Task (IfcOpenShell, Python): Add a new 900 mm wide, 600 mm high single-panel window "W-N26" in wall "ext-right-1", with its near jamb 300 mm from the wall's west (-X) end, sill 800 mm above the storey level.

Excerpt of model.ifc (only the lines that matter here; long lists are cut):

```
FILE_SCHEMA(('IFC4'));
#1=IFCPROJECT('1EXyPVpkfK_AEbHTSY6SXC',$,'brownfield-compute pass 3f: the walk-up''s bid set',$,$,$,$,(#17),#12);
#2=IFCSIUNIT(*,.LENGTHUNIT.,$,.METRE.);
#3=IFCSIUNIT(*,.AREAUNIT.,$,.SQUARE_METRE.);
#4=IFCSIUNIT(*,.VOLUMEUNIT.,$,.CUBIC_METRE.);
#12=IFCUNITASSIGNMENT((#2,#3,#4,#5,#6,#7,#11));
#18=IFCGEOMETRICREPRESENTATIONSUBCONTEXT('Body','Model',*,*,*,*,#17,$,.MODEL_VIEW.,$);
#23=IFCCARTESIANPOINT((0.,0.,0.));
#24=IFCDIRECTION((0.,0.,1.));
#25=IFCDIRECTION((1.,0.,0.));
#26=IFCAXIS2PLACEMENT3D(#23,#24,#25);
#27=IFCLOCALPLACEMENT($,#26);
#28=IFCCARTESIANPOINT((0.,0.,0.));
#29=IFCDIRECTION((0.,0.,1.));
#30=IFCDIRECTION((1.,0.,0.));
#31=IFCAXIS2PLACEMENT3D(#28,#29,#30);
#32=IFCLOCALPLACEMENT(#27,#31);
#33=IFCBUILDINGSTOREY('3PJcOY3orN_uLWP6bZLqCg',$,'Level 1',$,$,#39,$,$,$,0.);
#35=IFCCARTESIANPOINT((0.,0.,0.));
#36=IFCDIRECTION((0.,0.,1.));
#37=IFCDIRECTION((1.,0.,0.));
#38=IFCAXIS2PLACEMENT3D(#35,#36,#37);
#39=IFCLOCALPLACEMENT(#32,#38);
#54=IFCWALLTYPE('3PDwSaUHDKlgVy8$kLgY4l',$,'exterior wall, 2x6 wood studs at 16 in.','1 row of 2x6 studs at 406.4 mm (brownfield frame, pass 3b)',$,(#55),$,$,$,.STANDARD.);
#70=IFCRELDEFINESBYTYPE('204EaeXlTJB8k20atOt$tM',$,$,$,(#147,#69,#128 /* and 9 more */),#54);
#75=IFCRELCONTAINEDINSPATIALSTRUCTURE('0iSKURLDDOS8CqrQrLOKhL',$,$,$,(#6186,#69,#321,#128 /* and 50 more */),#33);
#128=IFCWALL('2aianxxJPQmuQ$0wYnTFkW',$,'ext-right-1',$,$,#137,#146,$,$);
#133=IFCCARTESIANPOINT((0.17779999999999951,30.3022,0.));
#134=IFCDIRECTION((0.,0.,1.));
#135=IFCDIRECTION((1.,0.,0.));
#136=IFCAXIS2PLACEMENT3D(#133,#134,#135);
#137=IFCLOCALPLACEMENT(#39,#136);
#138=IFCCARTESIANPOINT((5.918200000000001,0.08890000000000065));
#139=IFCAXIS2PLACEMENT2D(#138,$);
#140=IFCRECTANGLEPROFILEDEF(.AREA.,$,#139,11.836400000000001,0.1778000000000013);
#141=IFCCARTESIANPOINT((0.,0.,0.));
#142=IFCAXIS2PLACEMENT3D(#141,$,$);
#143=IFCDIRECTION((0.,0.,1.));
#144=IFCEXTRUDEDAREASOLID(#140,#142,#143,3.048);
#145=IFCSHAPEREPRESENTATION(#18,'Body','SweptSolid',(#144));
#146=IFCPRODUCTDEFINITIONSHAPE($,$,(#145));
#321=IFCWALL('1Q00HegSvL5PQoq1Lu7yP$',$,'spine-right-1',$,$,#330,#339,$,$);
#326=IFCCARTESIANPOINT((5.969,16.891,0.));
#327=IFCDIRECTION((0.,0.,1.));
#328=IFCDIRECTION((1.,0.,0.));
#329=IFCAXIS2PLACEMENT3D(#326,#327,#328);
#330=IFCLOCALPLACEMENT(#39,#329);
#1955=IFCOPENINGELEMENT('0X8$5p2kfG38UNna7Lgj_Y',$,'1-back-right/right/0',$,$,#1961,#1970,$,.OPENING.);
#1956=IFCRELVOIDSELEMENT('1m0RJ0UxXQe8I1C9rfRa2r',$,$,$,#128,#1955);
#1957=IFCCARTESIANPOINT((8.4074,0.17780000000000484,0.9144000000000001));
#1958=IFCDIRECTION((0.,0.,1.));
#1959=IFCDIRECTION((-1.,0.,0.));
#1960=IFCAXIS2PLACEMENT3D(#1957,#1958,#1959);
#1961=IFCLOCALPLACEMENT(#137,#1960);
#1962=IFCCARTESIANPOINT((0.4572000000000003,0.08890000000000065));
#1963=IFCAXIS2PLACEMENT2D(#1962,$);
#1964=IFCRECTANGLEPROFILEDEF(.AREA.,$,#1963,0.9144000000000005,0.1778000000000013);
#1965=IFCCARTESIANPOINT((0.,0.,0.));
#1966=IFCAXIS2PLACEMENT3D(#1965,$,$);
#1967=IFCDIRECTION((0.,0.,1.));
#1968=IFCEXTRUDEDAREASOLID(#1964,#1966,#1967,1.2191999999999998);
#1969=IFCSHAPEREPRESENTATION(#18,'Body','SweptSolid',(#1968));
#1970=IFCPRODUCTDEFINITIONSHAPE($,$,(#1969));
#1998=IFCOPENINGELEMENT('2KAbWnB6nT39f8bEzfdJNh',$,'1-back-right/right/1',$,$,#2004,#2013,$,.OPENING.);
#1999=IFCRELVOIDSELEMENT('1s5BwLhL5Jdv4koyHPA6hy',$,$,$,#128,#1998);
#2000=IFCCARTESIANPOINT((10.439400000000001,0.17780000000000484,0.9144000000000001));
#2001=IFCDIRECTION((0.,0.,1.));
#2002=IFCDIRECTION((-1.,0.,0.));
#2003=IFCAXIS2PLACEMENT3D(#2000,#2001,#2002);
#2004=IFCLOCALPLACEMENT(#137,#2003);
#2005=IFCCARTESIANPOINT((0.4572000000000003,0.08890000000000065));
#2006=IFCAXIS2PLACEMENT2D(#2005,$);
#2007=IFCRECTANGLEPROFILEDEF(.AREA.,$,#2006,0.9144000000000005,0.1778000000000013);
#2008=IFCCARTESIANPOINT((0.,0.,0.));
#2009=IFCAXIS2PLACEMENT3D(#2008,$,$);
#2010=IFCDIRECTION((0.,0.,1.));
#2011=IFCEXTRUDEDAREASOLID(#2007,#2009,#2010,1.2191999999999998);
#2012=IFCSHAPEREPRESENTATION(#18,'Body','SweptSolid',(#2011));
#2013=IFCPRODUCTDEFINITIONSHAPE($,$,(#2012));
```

```python
import numpy as np
import ifcopenshell
import ifcopenshell.api.feature
import ifcopenshell.api.geometry
import ifcopenshell.api.root
import ifcopenshell.api.spatial
import ifcopenshell.geom
import ifcopenshell.util.element
import ifcopenshell.util.placement
import ifcopenshell.util.representation
import ifcopenshell.util.shape
import ifcopenshell.util.unit

model = ifcopenshell.open("model.ifc")
unit_scale = ifcopenshell.util.unit.calculate_unit_scale(model)
settings = ifcopenshell.geom.settings()


def volume(element):
    """Net volume in cubic metres, openings subtracted."""
    shape = ifcopenshell.geom.create_shape(settings, element)
    return ifcopenshell.util.shape.get_volume(shape.geometry)


wall = model.by_guid("2aianxxJPQmuQ$0wYnTFkW")
storey = ifcopenshell.util.element.get_container(wall, ifc_class="IfcBuildingStorey")
context = ifcopenshell.util.representation.get_context(model, "Model", "Body", "MODEL_VIEW")
before = volume(wall)

width, height, from_end, sill = 0.9, 0.6, 0.3, 0.8  # metres

# The wall runs along its own X axis, and the end named is its -X end.
wall_shape = ifcopenshell.geom.create_shape(settings, wall)
x, y, z = ifcopenshell.util.shape.get_vertices(wall_shape.geometry).T
start = x.min() + from_end
face, thickness = float(y.min()), float(y.max() - y.min())
wall_matrix = ifcopenshell.util.placement.get_local_placement(wall.ObjectPlacement)
level = ifcopenshell.util.placement.get_local_placement(storey.ObjectPlacement)[2, 3]


def in_wall(x, y):
    """Placement at x, y metres in the wall's axes, at sill height."""
    matrix = wall_matrix.copy()
    matrix[:, 3] = wall_matrix @ np.array([x / unit_scale, y / unit_scale, 0.0, 1.0])
    matrix[2, 3] = level + sill / unit_scale
    return matrix


# Opening: a box that overshoots both wall faces by 50 mm.
opening = ifcopenshell.api.root.create_entity(model, ifc_class="IfcOpeningElement", predefined_type="OPENING")
box = ifcopenshell.api.geometry.add_wall_representation(
    model, context=context, length=width, height=height, thickness=thickness + 0.1
)
ifcopenshell.api.geometry.assign_representation(model, product=opening, representation=box)
ifcopenshell.api.geometry.edit_object_placement(model, product=opening, matrix=in_wall(start, face - 0.05), is_si=False)
ifcopenshell.api.feature.add_feature(model, feature=opening, element=wall)

window = ifcopenshell.api.root.create_entity(model, ifc_class="IfcWindow", name="W-N26", predefined_type="WINDOW")
window.OverallWidth, window.OverallHeight = width / unit_scale, height / unit_scale
window.PartitioningType = "SINGLE_PANEL"
body = ifcopenshell.api.geometry.add_window_representation(
    model,
    context=context,
    overall_width=window.OverallWidth,
    overall_height=window.OverallHeight,
    partition_type="SINGLE_PANEL",
)
ifcopenshell.api.geometry.assign_representation(model, product=window, representation=body)
ifcopenshell.api.spatial.assign_container(model, products=[window], relating_structure=storey)
ifcopenshell.api.feature.add_filling(model, opening=opening, element=window)

# Centre the window in the wall's thickness.
ifcopenshell.api.geometry.edit_object_placement(model, product=window, matrix=in_wall(start, face), is_si=False)
window_shape = ifcopenshell.geom.create_shape(settings, window)
depth = ifcopenshell.util.shape.get_vertices(window_shape.geometry)[:, 1]
offset = face + thickness / 2 - (depth.min() + depth.max()) / 2
ifcopenshell.api.geometry.edit_object_placement(model, product=window, matrix=in_wall(start, offset), is_si=False)

after = volume(wall)

print(f"wall volume {before:.3f} -> {after:.3f} m3")

model.write("model_edited.ifc")
```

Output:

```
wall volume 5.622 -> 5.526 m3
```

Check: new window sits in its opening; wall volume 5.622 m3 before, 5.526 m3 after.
